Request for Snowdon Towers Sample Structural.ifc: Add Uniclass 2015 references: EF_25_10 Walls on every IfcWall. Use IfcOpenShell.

First a look at what the model holds.

```python
import ifcopenshell

model = ifcopenshell.open("Snowdon Towers Sample Structural.ifc")
print(model.schema)
print("classifications:", [c.Name for c in model.by_type("IfcClassification")])
for ifc_class in ("IfcDoor", "IfcRoof", "IfcStair", "IfcWall", "IfcWindow"):
    print(ifc_class, len(model.by_type(ifc_class)))
```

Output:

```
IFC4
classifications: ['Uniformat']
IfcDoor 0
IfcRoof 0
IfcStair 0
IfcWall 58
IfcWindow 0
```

```python
import ifcopenshell
import ifcopenshell.api.classification

model = ifcopenshell.open("Snowdon Towers Sample Structural.ifc")

system = ifcopenshell.api.classification.add_classification(model, classification="Uniclass 2015")

codes = {
    "IfcWall": ("EF_25_10", "Walls"),
}
for ifc_class, (code, name) in codes.items():
    products = model.by_type(ifc_class)
    ifcopenshell.api.classification.add_reference(
        model, products=products, classification=system, identification=code, name=name
    )
    print(code, len(products))

model.write("Snowdon Towers Sample Structural-out.ifc")
```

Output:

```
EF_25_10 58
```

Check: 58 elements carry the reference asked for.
